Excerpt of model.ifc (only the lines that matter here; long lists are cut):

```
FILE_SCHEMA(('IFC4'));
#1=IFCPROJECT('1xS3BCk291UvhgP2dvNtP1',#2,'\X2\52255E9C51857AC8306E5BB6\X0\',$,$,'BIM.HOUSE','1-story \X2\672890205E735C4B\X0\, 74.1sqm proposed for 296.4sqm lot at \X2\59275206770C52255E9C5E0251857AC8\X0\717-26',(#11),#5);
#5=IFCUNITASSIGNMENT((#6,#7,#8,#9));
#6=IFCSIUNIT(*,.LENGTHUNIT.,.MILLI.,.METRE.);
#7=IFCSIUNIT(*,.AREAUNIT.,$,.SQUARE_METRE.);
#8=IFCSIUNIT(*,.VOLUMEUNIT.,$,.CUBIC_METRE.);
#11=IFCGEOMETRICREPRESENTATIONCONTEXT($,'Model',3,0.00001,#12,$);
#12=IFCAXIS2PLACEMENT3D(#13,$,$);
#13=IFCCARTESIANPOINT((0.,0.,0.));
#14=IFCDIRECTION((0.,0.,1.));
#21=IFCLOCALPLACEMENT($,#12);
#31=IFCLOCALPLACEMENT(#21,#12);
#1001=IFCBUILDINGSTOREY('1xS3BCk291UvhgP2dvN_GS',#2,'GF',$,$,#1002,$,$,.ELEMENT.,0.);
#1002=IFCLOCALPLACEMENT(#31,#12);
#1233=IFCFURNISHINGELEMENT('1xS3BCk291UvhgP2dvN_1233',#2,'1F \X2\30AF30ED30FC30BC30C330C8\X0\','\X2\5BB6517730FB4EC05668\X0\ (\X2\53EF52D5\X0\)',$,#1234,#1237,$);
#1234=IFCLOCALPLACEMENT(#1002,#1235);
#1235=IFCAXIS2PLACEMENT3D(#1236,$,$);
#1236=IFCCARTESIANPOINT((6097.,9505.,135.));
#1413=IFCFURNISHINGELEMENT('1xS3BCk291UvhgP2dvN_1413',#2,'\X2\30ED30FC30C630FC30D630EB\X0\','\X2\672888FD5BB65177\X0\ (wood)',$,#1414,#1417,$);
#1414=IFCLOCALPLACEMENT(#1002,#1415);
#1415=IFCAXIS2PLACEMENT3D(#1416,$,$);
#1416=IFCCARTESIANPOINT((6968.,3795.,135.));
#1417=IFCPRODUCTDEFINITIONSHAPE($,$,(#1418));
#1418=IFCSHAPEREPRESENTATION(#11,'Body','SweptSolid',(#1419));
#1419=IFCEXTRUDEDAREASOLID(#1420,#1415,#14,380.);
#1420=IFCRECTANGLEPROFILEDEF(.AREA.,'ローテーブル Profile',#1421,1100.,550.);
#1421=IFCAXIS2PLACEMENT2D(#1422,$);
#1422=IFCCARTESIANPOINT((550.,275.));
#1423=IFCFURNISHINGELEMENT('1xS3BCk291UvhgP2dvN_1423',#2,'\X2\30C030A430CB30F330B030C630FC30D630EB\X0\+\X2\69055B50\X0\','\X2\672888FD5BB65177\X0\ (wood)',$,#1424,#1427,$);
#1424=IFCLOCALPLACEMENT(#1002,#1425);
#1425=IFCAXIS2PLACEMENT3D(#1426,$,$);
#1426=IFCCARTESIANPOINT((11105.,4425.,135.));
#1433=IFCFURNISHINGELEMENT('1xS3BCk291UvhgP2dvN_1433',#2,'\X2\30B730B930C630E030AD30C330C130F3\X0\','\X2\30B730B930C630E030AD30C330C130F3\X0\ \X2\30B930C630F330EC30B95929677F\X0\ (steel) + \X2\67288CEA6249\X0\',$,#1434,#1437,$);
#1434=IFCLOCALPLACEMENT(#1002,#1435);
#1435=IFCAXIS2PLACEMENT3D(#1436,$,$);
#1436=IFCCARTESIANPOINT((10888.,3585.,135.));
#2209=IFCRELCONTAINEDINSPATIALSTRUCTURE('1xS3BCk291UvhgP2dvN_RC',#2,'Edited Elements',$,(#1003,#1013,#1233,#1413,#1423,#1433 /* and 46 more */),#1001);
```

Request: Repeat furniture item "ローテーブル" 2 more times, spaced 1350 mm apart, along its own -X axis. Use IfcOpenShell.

```python
import ifcopenshell
import ifcopenshell.api.geometry
import ifcopenshell.api.root
import ifcopenshell.util.element
import ifcopenshell.util.placement
import ifcopenshell.util.unit

model = ifcopenshell.open("model.ifc")
unit_scale = ifcopenshell.util.unit.calculate_unit_scale(model)


def reuse_history(source, copy):
    """copy_class also copies each property set's owner history, people and application; keep the originals."""
    for rel in copy.IsDefinedBy:
        if rel.is_a("IfcRelDefinesByProperties") and (history := rel.RelatingPropertyDefinition.OwnerHistory):
            rel.RelatingPropertyDefinition.OwnerHistory = source.OwnerHistory
            ifcopenshell.util.element.remove_deep2(model, history)


source = model.by_id(1413)
base = ifcopenshell.util.placement.get_local_placement(source.ObjectPlacement)
step = -base[:3, 0] * 1.35 / unit_scale

for i in range(1, 3):
    copy = ifcopenshell.api.root.copy_class(model, product=source)
    copy.Representation = ifcopenshell.util.element.copy_deep(
        model, source.Representation, exclude=["IfcGeometricRepresentationContext", "IfcRepresentationMap"]
    )
    reuse_history(source, copy)
    matrix = base.copy()
    matrix[:3, 3] += i * step
    print("added at", matrix[:3, 3].round(3) + 0.0)
    ifcopenshell.api.geometry.edit_object_placement(model, product=copy, matrix=matrix, is_si=False)

model.write("model-out.ifc")
```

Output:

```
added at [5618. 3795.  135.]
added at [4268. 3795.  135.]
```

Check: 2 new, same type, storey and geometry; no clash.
